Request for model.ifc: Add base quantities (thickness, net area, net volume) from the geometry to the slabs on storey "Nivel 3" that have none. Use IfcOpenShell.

First a look at what the model holds.

```python
import ifcopenshell
import ifcopenshell.util.element
import ifcopenshell.util.unit

model = ifcopenshell.open("model.ifc")
print(model.schema)
for unit_type in ("LENGTHUNIT", "AREAUNIT", "VOLUMEUNIT"):
    print(unit_type, ifcopenshell.util.unit.calculate_unit_scale(model, unit_type))
storey = next(s for s in model.by_type("IfcBuildingStorey") if s.Name == "Nivel 3")
slabs = [e for e in ifcopenshell.util.element.get_decomposition(storey) if e.is_a("IfcSlab")]
for e in sorted(slabs, key=lambda e: e.id()):
    print(e.id(), e.is_a(), e.Name, list(ifcopenshell.util.element.get_psets(e, qtos_only=True)), sep=" | ")
```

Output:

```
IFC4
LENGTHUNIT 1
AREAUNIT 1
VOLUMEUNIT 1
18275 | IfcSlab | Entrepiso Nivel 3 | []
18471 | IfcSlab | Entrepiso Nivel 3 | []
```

```python
import ifcopenshell
import ifcopenshell.api.pset
import ifcopenshell.geom
import ifcopenshell.util.element
import ifcopenshell.util.shape
import ifcopenshell.util.unit

model = ifcopenshell.open("model.ifc")
unit_scale = ifcopenshell.util.unit.calculate_unit_scale(model)
area_scale = ifcopenshell.util.unit.calculate_unit_scale(model, "AREAUNIT")
volume_scale = ifcopenshell.util.unit.calculate_unit_scale(model, "VOLUMEUNIT")
settings = ifcopenshell.geom.settings()

storey = next(s for s in model.by_type("IfcBuildingStorey") if s.Name == "Nivel 3")
slabs = [e for e in ifcopenshell.util.element.get_decomposition(storey) if e.is_a("IfcSlab")]

for e in sorted(slabs, key=lambda e: e.id()):
    if ifcopenshell.util.element.get_psets(e, qtos_only=True, should_inherit=False):
        continue
    # Geometry comes back in metres, in the element's own axes.
    shape = ifcopenshell.geom.create_shape(settings, e)
    values = {
        "Width": ifcopenshell.util.shape.get_z(shape.geometry) / unit_scale,
        "NetArea": ifcopenshell.util.shape.get_footprint_area(shape.geometry) / area_scale,
        "NetVolume": ifcopenshell.util.shape.get_volume(shape.geometry) / volume_scale,
    }
    qto = ifcopenshell.api.pset.add_qto(model, product=e, name="Qto_SlabBaseQuantities")
    ifcopenshell.api.pset.edit_qto(model, qto=qto, properties=values)
    print(e.id(), {k: round(v, 3) for k, v in values.items()})

model.write("model_edited.ifc")
```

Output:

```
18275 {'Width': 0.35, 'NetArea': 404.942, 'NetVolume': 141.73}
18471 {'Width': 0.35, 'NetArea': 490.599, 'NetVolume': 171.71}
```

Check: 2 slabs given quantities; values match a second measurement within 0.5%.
